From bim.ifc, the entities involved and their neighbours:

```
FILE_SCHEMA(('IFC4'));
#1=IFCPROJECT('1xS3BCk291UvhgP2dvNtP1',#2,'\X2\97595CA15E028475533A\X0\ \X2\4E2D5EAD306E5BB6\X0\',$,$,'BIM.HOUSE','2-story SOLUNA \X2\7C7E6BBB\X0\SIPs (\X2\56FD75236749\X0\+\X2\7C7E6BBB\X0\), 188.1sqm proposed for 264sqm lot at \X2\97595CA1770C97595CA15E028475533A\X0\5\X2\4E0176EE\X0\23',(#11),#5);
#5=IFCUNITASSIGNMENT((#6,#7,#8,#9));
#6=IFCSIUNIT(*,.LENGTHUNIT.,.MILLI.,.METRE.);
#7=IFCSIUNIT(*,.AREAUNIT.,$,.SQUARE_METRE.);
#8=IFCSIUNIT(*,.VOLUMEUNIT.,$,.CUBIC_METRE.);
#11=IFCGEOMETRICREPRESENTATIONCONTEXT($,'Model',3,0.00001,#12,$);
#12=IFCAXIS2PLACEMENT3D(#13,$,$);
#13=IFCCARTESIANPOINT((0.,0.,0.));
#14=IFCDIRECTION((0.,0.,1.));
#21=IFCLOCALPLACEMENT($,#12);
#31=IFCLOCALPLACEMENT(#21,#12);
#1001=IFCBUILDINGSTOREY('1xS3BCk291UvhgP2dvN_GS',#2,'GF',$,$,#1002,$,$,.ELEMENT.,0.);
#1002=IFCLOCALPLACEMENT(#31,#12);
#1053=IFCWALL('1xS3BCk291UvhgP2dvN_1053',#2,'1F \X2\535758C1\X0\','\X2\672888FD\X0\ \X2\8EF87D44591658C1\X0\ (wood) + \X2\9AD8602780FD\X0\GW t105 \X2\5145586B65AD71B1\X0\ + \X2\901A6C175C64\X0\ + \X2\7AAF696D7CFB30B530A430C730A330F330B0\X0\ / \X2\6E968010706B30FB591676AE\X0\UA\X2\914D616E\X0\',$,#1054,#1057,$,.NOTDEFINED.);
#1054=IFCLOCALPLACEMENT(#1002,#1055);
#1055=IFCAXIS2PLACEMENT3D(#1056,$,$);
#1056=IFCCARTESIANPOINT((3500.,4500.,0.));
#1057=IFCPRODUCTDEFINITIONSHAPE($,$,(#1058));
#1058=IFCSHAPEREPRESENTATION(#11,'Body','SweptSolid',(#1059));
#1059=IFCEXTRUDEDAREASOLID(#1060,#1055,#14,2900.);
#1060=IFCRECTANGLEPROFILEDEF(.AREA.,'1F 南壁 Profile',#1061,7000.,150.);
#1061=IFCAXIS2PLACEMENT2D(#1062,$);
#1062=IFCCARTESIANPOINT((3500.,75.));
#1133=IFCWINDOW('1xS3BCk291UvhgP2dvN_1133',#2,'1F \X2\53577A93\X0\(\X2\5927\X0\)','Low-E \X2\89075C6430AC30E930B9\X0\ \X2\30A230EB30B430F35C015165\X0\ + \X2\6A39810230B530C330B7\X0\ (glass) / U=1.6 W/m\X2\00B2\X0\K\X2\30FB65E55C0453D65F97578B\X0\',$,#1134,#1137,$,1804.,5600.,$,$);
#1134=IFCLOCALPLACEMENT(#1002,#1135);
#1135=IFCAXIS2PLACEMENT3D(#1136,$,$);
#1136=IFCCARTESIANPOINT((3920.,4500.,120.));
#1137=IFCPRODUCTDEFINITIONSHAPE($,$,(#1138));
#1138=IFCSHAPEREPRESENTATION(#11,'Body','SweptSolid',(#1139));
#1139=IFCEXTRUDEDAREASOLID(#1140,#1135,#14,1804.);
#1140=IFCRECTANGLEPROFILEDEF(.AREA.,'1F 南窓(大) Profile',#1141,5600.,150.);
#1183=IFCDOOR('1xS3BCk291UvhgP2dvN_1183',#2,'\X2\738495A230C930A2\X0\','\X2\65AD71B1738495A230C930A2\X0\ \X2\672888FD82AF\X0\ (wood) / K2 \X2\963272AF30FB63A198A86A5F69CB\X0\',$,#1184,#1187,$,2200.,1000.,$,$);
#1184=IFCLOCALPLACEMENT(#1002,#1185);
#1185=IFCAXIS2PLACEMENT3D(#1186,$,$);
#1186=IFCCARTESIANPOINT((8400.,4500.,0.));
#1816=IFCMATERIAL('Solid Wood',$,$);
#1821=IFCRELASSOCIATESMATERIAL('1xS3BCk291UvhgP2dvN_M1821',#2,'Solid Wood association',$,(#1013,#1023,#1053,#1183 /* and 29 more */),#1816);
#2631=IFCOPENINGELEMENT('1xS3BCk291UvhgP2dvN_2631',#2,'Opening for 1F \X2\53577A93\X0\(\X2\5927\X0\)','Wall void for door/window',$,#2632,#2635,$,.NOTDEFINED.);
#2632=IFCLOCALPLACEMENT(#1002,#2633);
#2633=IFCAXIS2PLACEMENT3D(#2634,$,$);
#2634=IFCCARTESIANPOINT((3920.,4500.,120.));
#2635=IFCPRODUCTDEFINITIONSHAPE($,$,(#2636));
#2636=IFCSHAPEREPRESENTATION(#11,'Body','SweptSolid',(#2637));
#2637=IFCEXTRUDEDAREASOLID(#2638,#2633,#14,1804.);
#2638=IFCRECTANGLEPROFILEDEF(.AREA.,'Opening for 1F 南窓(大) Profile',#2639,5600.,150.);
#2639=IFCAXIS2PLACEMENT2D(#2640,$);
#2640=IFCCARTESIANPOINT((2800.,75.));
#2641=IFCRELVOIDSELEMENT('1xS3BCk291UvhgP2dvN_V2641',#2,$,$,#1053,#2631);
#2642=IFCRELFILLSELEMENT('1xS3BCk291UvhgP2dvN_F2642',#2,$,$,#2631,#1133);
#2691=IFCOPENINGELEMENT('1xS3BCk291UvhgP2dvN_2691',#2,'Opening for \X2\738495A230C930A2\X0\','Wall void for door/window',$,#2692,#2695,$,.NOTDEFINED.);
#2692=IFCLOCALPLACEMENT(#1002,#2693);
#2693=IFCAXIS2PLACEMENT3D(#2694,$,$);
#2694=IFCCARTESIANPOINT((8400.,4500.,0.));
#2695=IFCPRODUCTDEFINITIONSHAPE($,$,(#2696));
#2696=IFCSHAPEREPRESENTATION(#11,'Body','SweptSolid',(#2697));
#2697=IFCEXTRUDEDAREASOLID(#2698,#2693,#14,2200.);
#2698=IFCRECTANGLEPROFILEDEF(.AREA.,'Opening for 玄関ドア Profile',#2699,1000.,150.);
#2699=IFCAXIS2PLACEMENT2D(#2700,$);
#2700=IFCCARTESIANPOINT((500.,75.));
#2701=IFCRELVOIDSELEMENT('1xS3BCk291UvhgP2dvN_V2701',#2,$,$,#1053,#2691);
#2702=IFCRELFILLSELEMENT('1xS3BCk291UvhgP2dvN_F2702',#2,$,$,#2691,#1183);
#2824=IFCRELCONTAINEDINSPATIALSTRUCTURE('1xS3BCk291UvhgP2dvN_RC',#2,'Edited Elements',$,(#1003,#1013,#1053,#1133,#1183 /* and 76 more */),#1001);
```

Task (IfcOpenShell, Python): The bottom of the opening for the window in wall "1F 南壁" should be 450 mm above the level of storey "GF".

```python
import numpy as np
import ifcopenshell
import ifcopenshell.api.geometry
import ifcopenshell.geom
import ifcopenshell.util.element
import ifcopenshell.util.placement
import ifcopenshell.util.shape
import ifcopenshell.util.unit

model = ifcopenshell.open("bim.ifc")
unit_scale = ifcopenshell.util.unit.calculate_unit_scale(model)

window = model.by_guid("1xS3BCk291UvhgP2dvN_1133")
opening = window.FillsVoids[0].RelatingOpeningElement
storey = ifcopenshell.util.element.get_container(window, ifc_class="IfcBuildingStorey")
level = ifcopenshell.util.placement.get_local_placement(storey.ObjectPlacement)[2, 3]

# The opening's origin need not be at the sill, so measure its lowest point.
shape = ifcopenshell.geom.create_shape(ifcopenshell.geom.settings(), opening)
bottom = ifcopenshell.util.shape.get_shape_bottom_elevation(shape, shape.geometry) / unit_scale
dz = level + 0.45 / unit_scale - bottom

shift = np.array([0.0, 0.0, dz])
# The window is not placed relative to its opening, so move both.
for product in (opening, window):
    matrix = ifcopenshell.util.placement.get_local_placement(product.ObjectPlacement)
    matrix[:3, 3] += shift
    ifcopenshell.api.geometry.edit_object_placement(model, product=product, matrix=matrix, is_si=False)

print(f"moved by {dz * unit_scale:+.3f} m")

model.write("bim_rev.ifc")
```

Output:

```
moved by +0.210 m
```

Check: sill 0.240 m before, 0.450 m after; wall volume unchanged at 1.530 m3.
